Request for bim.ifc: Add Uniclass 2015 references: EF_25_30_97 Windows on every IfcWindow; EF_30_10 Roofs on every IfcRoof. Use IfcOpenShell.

First a look at what the model holds.

```python
import ifcopenshell

model = ifcopenshell.open("bim.ifc")
print(model.schema)
print("classifications:", [c.Name for c in model.by_type("IfcClassification")])
for ifc_class in ("IfcDoor", "IfcRoof", "IfcStair", "IfcWall", "IfcWindow"):
    print(ifc_class, len(model.by_type(ifc_class)))
```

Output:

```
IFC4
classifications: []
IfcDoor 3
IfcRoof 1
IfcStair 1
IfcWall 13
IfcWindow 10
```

```python
import ifcopenshell
import ifcopenshell.api.classification

model = ifcopenshell.open("bim.ifc")

system = ifcopenshell.api.classification.add_classification(model, classification="Uniclass 2015")

codes = {
    "IfcWindow": ("EF_25_30_97", "Windows"),
    "IfcRoof": ("EF_30_10", "Roofs"),
}
for ifc_class, (code, name) in codes.items():
    products = model.by_type(ifc_class)
    ifcopenshell.api.classification.add_reference(
        model, products=products, classification=system, identification=code, name=name
    )
    print(code, len(products))

model.write("bim_rev.ifc")
```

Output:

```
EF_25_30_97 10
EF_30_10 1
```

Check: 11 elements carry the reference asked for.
